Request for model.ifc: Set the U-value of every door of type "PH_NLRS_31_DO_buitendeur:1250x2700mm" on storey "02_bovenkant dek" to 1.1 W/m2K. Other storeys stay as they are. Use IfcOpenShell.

First a look at what the model holds.

```python
import ifcopenshell
import ifcopenshell.util.element

model = ifcopenshell.open("model.ifc")
print(model.schema)
storey = next(s for s in model.by_type("IfcBuildingStorey") if s.Name == "02_bovenkant dek")
doors = [e for e in ifcopenshell.util.element.get_decomposition(storey) if e.is_a("IfcDoor")]
seen = {}
for e in doors:
    element_type = ifcopenshell.util.element.get_type(e)
    key = (element_type.Name if element_type != e and element_type else None, ifcopenshell.util.element.get_pset(e, "Pset_DoorCommon", "ThermalTransmittance"))
    seen[key] = seen.get(key, 0) + 1
for (name, value), count in sorted(seen.items(), key=str):
    print(count, "x", name, "|", value)
```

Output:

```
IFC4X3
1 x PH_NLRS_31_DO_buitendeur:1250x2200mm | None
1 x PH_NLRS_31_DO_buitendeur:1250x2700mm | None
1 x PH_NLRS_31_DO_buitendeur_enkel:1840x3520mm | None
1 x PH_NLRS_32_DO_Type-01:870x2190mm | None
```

```python
import ifcopenshell
import ifcopenshell.api.pset
import ifcopenshell.util.element

model = ifcopenshell.open("model.ifc")

storey = next(s for s in model.by_type("IfcBuildingStorey") if s.Name == "02_bovenkant dek")
doors = [e for e in ifcopenshell.util.element.get_decomposition(storey) if e.is_a("IfcDoor")]

count = 0
for e in doors:
    element_type = ifcopenshell.util.element.get_type(e)
    if element_type in (None, e) or element_type.Name != "PH_NLRS_31_DO_buitendeur:1250x2700mm":
        continue
    # add_pset returns the element's existing set when there is one.
    pset = ifcopenshell.api.pset.add_pset(model, product=e, name="Pset_DoorCommon")
    ifcopenshell.api.pset.edit_pset(model, pset=pset, properties={"ThermalTransmittance": 1.1})
    count += 1

print(count, "doors updated")

model.write("model_rev.ifc")
```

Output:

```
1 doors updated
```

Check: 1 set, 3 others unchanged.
